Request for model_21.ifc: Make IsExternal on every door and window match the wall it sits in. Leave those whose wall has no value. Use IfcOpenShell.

First a look at what the model holds.

```python
import ifcopenshell
import ifcopenshell.util.element

model = ifcopenshell.open("model_21.ifc")
print(model.schema)
seen = {}
for e in model.by_type("IfcDoor") + model.by_type("IfcWindow"):
    if not e.FillsVoids:
        continue
    host = e.FillsVoids[0].RelatingOpeningElement.VoidsElements[0].RelatingBuildingElement
    own = ifcopenshell.util.element.get_pset(e, f"Pset_{e.is_a()[3:].removesuffix('StandardCase')}Common", "IsExternal")
    wall = ifcopenshell.util.element.get_pset(host, "Pset_WallCommon", "IsExternal")
    seen[e.is_a(), own, wall] = seen.get((e.is_a(), own, wall), 0) + 1
for (cls, own, wall), count in sorted(seen.items(), key=str):
    print(count, cls, "IsExternal:", own, "| host wall:", wall)
```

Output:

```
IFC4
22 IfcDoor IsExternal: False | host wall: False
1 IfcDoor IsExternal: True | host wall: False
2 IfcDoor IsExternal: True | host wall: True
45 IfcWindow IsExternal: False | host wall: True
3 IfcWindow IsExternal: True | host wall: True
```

```python
import ifcopenshell
import ifcopenshell.api.pset
import ifcopenshell.util.element

model = ifcopenshell.open("model_21.ifc")

count = 0
for ifc_class, pset_name in (("IfcDoor", "Pset_DoorCommon"), ("IfcWindow", "Pset_WindowCommon")):
    for e in model.by_type(ifc_class):
        if not e.FillsVoids:
            continue
        host = e.FillsVoids[0].RelatingOpeningElement.VoidsElements[0].RelatingBuildingElement
        external = ifcopenshell.util.element.get_pset(host, "Pset_WallCommon", "IsExternal")
        if external is None or ifcopenshell.util.element.get_pset(e, pset_name, "IsExternal") == external:
            continue
        pset = ifcopenshell.api.pset.add_pset(model, product=e, name=pset_name)
        ifcopenshell.api.pset.edit_pset(model, pset=pset, properties={"IsExternal": external})
        count += 1

print(count, "updated")

model.write("model_21-out.ifc")
```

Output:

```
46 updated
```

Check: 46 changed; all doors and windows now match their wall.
